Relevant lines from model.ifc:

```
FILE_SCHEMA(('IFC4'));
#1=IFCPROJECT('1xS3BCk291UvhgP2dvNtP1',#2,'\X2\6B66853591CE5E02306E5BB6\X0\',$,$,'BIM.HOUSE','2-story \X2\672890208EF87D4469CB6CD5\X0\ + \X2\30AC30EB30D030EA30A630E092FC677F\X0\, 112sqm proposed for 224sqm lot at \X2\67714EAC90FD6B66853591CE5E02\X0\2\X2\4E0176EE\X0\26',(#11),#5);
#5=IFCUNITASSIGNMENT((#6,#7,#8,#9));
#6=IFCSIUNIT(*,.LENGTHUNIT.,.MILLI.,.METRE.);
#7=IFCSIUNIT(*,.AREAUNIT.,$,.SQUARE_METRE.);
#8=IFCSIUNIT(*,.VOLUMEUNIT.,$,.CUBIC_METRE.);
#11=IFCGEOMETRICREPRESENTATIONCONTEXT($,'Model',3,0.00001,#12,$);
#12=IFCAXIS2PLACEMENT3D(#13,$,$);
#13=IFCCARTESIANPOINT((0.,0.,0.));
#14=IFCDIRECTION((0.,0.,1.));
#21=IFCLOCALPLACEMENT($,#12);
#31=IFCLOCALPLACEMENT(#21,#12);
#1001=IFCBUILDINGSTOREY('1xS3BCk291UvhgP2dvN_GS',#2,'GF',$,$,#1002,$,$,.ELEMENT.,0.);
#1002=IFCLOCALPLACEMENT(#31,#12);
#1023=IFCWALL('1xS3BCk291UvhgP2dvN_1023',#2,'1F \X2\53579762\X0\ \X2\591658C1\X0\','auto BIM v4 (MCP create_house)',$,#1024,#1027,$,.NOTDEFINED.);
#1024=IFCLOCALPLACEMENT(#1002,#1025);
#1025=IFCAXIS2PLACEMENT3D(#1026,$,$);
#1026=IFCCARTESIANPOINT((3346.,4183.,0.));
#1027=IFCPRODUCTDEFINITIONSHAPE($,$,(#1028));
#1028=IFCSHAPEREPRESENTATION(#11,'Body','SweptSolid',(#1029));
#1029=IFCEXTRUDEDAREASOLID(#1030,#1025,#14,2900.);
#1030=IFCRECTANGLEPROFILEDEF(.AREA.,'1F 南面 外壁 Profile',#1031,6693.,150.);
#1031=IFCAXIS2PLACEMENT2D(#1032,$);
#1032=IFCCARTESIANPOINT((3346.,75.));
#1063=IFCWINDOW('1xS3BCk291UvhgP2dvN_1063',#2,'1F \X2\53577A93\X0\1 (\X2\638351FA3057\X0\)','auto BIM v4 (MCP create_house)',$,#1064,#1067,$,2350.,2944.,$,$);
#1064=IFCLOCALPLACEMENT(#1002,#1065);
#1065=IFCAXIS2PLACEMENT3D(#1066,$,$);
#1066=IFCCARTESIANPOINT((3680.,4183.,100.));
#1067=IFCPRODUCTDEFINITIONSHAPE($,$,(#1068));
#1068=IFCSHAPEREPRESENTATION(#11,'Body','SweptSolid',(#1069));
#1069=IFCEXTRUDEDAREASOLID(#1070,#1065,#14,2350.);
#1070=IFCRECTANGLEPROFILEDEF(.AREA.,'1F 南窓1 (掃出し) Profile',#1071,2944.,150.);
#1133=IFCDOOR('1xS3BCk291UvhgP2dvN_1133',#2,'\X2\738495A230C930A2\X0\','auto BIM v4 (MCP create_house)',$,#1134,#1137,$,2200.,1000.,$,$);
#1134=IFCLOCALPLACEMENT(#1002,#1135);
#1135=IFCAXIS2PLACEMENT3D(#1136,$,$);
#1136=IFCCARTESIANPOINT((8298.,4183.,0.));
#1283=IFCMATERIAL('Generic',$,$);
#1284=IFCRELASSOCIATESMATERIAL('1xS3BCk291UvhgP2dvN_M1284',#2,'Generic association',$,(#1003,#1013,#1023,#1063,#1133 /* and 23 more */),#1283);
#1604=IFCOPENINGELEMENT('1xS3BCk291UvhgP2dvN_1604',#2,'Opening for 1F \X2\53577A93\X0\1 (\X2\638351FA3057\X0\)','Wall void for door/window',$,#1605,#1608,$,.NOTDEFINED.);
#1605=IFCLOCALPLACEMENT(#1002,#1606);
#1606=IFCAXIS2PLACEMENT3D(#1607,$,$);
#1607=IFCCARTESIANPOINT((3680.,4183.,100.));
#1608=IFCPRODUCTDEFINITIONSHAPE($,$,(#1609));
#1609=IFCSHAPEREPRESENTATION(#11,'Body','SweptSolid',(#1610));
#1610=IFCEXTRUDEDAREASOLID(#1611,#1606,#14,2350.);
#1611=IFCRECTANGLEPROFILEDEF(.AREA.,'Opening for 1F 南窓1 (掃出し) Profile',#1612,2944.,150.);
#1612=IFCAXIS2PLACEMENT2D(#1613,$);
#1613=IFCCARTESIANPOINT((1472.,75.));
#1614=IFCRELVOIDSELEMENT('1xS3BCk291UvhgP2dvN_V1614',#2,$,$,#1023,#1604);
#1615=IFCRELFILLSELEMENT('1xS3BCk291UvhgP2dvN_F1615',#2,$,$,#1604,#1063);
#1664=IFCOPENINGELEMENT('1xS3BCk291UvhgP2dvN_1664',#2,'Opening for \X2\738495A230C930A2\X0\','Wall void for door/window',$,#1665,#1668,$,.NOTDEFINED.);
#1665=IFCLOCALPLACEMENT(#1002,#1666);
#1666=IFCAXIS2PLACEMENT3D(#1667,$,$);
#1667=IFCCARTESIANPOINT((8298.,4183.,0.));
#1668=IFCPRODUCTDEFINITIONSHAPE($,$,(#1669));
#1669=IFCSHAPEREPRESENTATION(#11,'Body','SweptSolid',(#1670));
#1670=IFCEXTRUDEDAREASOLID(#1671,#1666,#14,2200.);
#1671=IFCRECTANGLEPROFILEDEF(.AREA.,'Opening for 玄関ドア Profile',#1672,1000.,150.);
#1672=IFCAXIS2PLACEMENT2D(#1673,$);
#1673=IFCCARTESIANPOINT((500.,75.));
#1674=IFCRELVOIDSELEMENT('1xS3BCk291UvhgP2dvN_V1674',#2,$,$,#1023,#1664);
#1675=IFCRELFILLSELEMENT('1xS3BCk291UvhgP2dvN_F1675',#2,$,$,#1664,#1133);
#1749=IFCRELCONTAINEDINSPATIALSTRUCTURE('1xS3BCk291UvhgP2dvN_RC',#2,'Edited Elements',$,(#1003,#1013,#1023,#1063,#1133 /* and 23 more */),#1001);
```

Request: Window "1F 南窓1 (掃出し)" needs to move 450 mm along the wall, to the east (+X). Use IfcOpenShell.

```python
import ifcopenshell
import ifcopenshell.api.geometry
import ifcopenshell.util.placement

model = ifcopenshell.open("model.ifc")

window = model.by_guid("1xS3BCk291UvhgP2dvN_1063")
opening = window.FillsVoids[0].RelatingOpeningElement
wall = opening.VoidsElements[0].RelatingBuildingElement

wall_matrix = ifcopenshell.util.placement.get_local_placement(wall.ObjectPlacement)
shift = wall_matrix[:3, 0] * 450.0
before = ifcopenshell.util.placement.get_local_placement(window.ObjectPlacement)[:3, 3].copy()

# The window is not placed relative to its opening, so move both.
for product in (opening, window):
    matrix = ifcopenshell.util.placement.get_local_placement(product.ObjectPlacement)
    matrix[:3, 3] += shift
    ifcopenshell.api.geometry.edit_object_placement(model, product=product, matrix=matrix, is_si=False)

after = ifcopenshell.util.placement.get_local_placement(window.ObjectPlacement)[:3, 3]
print("window moved by", (after - before).round(3) + 0.0)

model.write("model_v2.ifc")
```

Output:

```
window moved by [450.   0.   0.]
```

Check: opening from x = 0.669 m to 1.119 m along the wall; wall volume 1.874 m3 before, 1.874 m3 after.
